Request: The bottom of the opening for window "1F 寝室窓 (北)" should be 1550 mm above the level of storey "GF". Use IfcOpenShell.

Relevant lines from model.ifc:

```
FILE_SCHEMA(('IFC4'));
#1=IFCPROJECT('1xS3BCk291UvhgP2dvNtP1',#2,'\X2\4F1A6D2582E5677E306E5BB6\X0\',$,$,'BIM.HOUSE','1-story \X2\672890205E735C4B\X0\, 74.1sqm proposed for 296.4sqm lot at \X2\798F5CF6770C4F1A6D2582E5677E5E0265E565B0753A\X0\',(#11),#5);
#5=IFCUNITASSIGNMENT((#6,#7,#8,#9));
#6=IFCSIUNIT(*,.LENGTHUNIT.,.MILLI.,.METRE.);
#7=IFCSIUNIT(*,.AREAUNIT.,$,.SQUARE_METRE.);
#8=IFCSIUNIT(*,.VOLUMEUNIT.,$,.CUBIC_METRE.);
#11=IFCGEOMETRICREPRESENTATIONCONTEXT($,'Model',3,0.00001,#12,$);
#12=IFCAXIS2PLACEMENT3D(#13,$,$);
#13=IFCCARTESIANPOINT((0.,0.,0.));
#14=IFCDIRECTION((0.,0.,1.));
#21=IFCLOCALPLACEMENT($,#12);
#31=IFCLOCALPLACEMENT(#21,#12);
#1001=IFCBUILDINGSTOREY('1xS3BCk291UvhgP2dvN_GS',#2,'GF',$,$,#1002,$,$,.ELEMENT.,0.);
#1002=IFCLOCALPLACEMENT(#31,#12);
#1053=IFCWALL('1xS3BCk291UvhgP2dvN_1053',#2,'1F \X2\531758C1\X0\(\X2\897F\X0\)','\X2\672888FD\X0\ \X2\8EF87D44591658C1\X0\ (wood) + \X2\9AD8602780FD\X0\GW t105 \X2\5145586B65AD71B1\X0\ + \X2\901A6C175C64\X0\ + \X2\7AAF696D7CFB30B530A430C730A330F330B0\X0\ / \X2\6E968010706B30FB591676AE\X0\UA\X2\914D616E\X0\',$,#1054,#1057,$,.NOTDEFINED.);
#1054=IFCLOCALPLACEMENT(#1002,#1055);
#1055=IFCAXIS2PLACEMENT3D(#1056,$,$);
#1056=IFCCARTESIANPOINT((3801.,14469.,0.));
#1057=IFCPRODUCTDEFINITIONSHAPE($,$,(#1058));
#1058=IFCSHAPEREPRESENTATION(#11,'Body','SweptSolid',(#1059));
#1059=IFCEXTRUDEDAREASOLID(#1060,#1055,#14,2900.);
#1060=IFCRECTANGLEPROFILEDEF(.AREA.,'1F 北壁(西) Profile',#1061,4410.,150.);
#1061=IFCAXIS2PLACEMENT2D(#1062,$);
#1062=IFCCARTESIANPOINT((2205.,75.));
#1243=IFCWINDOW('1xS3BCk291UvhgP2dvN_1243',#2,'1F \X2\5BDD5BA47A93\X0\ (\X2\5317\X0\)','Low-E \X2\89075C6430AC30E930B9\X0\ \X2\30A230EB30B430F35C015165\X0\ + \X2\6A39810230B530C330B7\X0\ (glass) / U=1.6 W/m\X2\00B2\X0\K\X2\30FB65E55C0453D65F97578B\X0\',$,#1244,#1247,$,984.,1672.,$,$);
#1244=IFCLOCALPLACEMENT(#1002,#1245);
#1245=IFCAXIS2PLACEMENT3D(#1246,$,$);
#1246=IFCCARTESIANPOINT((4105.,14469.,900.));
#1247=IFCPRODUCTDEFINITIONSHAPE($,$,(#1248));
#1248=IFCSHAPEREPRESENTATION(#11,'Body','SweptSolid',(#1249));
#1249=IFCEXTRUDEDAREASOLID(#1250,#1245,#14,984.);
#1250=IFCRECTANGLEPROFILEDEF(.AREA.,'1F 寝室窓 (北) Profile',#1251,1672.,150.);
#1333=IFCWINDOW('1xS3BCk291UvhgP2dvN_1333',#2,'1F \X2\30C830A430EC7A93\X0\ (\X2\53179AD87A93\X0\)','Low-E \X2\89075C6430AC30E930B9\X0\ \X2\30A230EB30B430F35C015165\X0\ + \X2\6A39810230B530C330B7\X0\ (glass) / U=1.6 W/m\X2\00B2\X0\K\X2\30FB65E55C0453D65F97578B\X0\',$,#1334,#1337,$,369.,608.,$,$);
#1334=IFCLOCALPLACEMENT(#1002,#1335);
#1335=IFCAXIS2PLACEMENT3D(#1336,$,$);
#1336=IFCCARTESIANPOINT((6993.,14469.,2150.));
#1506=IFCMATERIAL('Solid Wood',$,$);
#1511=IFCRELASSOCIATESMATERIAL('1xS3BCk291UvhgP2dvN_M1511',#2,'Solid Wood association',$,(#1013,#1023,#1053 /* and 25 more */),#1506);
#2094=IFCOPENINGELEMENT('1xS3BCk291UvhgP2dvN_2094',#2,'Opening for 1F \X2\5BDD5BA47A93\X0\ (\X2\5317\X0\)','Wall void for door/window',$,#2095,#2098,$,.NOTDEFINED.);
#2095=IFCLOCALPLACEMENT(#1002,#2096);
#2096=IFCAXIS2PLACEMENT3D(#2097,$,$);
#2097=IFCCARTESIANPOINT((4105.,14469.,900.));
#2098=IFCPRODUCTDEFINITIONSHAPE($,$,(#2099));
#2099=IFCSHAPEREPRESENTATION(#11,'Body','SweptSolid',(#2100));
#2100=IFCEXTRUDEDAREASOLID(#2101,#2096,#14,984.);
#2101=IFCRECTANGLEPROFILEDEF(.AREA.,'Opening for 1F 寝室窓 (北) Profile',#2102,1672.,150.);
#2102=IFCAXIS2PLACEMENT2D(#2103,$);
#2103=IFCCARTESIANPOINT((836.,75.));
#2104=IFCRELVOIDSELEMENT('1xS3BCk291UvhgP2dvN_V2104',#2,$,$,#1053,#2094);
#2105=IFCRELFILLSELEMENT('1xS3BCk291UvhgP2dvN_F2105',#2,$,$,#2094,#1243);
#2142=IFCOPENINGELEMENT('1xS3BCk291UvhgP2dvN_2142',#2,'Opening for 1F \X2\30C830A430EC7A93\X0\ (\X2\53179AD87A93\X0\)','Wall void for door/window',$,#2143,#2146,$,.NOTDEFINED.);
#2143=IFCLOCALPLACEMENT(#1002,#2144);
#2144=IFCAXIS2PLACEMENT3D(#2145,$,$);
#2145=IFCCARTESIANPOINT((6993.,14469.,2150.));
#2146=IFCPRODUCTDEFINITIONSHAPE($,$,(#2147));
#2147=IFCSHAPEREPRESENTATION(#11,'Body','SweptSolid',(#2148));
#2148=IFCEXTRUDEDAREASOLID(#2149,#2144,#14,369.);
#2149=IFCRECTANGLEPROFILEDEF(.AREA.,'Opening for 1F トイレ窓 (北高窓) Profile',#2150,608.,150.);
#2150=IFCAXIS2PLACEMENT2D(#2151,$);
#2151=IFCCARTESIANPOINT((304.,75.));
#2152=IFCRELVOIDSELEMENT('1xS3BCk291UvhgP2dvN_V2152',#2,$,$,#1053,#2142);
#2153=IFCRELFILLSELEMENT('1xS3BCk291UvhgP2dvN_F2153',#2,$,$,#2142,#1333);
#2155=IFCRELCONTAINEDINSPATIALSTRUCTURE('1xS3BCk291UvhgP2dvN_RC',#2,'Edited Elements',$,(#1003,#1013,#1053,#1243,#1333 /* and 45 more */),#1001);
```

```python
import numpy as np
import ifcopenshell
import ifcopenshell.api.geometry
import ifcopenshell.geom
import ifcopenshell.util.element
import ifcopenshell.util.placement
import ifcopenshell.util.shape
import ifcopenshell.util.unit

model = ifcopenshell.open("model.ifc")
unit_scale = ifcopenshell.util.unit.calculate_unit_scale(model)

window = model.by_guid("1xS3BCk291UvhgP2dvN_1243")
opening = window.FillsVoids[0].RelatingOpeningElement
storey = ifcopenshell.util.element.get_container(window, ifc_class="IfcBuildingStorey")
level = ifcopenshell.util.placement.get_local_placement(storey.ObjectPlacement)[2, 3]

# The opening's origin need not be at the sill, so measure its lowest point.
shape = ifcopenshell.geom.create_shape(ifcopenshell.geom.settings(), opening)
bottom = ifcopenshell.util.shape.get_shape_bottom_elevation(shape, shape.geometry) / unit_scale
dz = level + 1.55 / unit_scale - bottom

shift = np.array([0.0, 0.0, dz])
# The window is not placed relative to its opening, so move both.
for product in (opening, window):
    matrix = ifcopenshell.util.placement.get_local_placement(product.ObjectPlacement)
    matrix[:3, 3] += shift
    ifcopenshell.api.geometry.edit_object_placement(model, product=product, matrix=matrix, is_si=False)

print(f"moved by {dz * unit_scale:+.3f} m")

model.write("model_edited.ifc")
```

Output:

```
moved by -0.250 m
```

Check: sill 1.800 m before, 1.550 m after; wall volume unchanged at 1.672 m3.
